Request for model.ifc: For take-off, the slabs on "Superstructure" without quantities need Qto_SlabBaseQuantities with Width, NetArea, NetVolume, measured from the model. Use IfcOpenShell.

First a look at what the model holds.

```python
import ifcopenshell
import ifcopenshell.util.element
import ifcopenshell.util.unit

model = ifcopenshell.open("model.ifc")
print(model.schema)
for unit_type in ("LENGTHUNIT", "AREAUNIT", "VOLUMEUNIT"):
    print(unit_type, ifcopenshell.util.unit.calculate_unit_scale(model, unit_type))
storey = next(s for s in model.by_type("IfcBuildingStorey") if s.Name == "Superstructure")
slabs = [e for e in ifcopenshell.util.element.get_decomposition(storey) if e.is_a("IfcSlab")]
for e in sorted(slabs, key=lambda e: e.id()):
    print(e.id(), e.is_a(), e.Name, list(ifcopenshell.util.element.get_psets(e, qtos_only=True)), sep=" | ")
```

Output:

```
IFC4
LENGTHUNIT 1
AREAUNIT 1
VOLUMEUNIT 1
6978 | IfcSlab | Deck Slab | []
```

```python
import ifcopenshell
import ifcopenshell.api.pset
import ifcopenshell.geom
import ifcopenshell.util.element
import ifcopenshell.util.shape
import ifcopenshell.util.unit

model = ifcopenshell.open("model.ifc")
unit_scale = ifcopenshell.util.unit.calculate_unit_scale(model)
area_scale = ifcopenshell.util.unit.calculate_unit_scale(model, "AREAUNIT")
volume_scale = ifcopenshell.util.unit.calculate_unit_scale(model, "VOLUMEUNIT")
settings = ifcopenshell.geom.settings()

storey = next(s for s in model.by_type("IfcBuildingStorey") if s.Name == "Superstructure")
slabs = [e for e in ifcopenshell.util.element.get_decomposition(storey) if e.is_a("IfcSlab")]

for e in sorted(slabs, key=lambda e: e.id()):
    if ifcopenshell.util.element.get_psets(e, qtos_only=True, should_inherit=False):
        continue
    # Geometry comes back in metres, in the element's own axes.
    shape = ifcopenshell.geom.create_shape(settings, e)
    values = {
        "Width": ifcopenshell.util.shape.get_z(shape.geometry) / unit_scale,
        "NetArea": ifcopenshell.util.shape.get_footprint_area(shape.geometry) / area_scale,
        "NetVolume": ifcopenshell.util.shape.get_volume(shape.geometry) / volume_scale,
    }
    qto = ifcopenshell.api.pset.add_qto(model, product=e, name="Qto_SlabBaseQuantities")
    ifcopenshell.api.pset.edit_qto(model, qto=qto, properties=values)
    print(e.id(), {k: round(v, 3) for k, v in values.items()})

model.write("model-out.ifc")
```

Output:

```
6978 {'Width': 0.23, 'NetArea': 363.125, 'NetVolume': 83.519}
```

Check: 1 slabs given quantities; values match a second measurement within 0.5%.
